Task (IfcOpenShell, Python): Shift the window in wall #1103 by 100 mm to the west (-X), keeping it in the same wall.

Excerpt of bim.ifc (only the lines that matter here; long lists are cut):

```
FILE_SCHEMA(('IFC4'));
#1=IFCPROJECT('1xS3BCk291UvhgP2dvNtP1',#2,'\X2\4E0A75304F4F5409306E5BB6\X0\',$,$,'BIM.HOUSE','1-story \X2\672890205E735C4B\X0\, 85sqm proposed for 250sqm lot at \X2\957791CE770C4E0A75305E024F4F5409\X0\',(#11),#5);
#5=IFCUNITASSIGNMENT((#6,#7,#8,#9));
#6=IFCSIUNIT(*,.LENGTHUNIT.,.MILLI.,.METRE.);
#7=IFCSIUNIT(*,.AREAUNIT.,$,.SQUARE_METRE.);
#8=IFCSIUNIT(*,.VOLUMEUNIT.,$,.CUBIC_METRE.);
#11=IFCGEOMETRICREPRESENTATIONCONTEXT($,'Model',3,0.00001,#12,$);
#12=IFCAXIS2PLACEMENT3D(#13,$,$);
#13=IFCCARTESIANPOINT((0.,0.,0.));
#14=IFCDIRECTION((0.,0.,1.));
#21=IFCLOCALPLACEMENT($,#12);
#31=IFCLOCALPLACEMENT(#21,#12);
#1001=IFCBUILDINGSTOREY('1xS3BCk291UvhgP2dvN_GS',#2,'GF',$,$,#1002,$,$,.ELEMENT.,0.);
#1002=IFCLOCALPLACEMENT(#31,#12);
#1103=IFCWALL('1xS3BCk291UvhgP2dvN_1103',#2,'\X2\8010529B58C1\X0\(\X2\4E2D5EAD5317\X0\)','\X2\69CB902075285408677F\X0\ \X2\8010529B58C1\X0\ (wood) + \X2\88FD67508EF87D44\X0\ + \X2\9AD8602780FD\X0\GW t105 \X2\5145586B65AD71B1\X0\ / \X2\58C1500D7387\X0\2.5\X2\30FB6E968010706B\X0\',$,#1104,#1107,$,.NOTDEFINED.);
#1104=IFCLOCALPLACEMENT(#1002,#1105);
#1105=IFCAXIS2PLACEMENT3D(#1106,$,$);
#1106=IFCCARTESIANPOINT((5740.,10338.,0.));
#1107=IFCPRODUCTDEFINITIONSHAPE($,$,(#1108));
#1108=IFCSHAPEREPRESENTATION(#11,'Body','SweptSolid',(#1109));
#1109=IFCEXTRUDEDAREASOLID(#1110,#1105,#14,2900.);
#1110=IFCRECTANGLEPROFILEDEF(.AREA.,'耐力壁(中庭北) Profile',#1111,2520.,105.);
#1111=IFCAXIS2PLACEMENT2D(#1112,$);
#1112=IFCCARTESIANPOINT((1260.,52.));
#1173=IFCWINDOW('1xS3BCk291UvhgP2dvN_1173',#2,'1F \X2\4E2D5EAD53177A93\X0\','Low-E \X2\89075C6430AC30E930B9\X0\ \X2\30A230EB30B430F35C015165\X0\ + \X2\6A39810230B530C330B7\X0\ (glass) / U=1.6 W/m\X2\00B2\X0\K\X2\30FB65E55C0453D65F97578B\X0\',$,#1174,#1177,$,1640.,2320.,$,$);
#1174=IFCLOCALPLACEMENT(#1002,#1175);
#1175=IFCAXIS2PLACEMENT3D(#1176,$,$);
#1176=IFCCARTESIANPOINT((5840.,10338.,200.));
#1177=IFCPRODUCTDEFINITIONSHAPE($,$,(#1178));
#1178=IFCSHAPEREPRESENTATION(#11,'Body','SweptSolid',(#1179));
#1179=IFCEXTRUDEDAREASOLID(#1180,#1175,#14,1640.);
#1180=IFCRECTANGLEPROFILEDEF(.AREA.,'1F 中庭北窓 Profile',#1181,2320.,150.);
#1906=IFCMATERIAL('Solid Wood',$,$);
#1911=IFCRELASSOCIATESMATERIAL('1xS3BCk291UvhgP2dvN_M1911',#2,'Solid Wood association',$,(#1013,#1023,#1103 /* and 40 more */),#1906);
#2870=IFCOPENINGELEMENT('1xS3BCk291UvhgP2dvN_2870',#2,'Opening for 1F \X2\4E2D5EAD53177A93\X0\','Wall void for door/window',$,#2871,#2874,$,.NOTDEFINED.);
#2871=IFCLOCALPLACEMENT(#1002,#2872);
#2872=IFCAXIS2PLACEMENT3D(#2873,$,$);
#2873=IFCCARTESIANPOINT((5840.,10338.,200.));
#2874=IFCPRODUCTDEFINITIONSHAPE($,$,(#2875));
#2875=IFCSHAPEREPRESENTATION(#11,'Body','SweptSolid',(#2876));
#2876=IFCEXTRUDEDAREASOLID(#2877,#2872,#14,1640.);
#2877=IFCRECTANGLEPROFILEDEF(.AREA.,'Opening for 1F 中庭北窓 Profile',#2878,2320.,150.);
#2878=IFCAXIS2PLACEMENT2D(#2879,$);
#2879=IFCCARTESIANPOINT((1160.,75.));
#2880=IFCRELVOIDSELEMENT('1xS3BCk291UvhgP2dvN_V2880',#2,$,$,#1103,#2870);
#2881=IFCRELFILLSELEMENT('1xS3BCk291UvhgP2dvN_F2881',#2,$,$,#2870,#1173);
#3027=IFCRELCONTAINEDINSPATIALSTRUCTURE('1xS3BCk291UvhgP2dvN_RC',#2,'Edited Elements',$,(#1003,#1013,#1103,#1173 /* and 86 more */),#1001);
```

```python
import ifcopenshell
import ifcopenshell.api.geometry
import ifcopenshell.util.placement
import ifcopenshell.util.unit

model = ifcopenshell.open("bim.ifc")
unit_scale = ifcopenshell.util.unit.calculate_unit_scale(model)

window = model.by_guid("1xS3BCk291UvhgP2dvN_1173")
opening = window.FillsVoids[0].RelatingOpeningElement
wall = opening.VoidsElements[0].RelatingBuildingElement

wall_matrix = ifcopenshell.util.placement.get_local_placement(wall.ObjectPlacement)
shift = wall_matrix[:3, 0] * -0.1 / unit_scale
before = ifcopenshell.util.placement.get_local_placement(window.ObjectPlacement)[:3, 3].copy()

# The window is not placed relative to its opening, so move both.
for product in (opening, window):
    matrix = ifcopenshell.util.placement.get_local_placement(product.ObjectPlacement)
    matrix[:3, 3] += shift
    ifcopenshell.api.geometry.edit_object_placement(model, product=product, matrix=matrix, is_si=False)

after = ifcopenshell.util.placement.get_local_placement(window.ObjectPlacement)[:3, 3]
print("window moved by", (after - before).round(3) + 0.0)

model.write("bim_rev.ifc")
```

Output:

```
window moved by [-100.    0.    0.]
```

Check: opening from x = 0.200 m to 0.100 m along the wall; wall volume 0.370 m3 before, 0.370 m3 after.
